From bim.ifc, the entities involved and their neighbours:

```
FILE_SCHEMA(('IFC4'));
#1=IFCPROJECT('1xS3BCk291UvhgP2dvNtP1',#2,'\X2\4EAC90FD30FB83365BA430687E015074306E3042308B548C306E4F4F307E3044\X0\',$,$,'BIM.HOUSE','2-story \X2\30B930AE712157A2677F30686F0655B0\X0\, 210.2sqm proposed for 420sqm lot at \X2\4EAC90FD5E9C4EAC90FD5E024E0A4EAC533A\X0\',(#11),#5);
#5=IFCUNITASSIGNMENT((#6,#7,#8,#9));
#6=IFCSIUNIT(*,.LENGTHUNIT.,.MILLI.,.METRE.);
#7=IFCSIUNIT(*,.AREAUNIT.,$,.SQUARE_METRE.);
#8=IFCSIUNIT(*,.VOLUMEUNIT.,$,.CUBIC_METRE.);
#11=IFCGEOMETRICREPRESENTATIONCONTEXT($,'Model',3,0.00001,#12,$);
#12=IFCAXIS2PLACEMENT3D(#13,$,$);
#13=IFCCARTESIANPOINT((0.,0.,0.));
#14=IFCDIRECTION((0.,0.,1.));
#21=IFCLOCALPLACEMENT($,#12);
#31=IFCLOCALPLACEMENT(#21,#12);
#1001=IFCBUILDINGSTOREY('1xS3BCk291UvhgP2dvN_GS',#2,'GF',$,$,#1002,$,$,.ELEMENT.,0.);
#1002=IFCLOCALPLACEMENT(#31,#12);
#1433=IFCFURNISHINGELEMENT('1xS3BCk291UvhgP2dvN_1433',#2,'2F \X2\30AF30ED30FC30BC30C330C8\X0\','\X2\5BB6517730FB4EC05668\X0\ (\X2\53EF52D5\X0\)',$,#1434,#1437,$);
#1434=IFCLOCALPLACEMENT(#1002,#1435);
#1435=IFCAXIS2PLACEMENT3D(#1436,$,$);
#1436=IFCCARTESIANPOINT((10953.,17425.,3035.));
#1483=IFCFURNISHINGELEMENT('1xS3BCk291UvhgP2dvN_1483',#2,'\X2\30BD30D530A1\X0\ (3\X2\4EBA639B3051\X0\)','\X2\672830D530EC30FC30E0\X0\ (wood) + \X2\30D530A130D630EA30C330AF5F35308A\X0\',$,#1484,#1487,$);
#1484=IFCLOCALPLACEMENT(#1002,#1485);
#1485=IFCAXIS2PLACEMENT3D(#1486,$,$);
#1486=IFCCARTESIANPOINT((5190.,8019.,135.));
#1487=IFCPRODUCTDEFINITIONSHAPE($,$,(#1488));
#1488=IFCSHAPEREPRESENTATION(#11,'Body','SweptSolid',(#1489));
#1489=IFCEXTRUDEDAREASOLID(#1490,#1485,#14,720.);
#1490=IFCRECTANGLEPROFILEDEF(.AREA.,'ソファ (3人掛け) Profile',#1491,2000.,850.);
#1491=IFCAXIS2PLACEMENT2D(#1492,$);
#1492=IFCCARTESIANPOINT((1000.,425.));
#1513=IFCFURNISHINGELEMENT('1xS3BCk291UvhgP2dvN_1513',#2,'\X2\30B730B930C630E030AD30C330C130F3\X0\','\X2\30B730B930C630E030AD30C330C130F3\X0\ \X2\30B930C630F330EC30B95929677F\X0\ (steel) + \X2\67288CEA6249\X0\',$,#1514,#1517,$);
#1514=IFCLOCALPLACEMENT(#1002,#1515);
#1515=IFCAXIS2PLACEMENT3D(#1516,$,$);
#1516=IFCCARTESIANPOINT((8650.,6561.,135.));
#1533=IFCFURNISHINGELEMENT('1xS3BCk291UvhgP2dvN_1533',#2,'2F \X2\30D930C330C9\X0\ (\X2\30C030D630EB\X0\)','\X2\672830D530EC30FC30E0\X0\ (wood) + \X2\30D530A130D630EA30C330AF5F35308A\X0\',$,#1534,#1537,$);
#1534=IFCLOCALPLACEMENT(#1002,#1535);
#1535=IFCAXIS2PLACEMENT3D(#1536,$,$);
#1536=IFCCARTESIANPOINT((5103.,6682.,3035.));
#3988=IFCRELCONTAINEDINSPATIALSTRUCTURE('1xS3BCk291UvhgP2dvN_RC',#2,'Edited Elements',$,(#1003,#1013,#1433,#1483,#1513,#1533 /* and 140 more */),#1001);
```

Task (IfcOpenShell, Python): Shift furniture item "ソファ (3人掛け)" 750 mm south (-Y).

```python
import ifcopenshell
import ifcopenshell.api.geometry
import ifcopenshell.util.placement

model = ifcopenshell.open("bim.ifc")

item = model.by_id(1483)
matrix = ifcopenshell.util.placement.get_local_placement(item.ObjectPlacement)
matrix[1, 3] -= 750.0
ifcopenshell.api.geometry.edit_object_placement(model, product=item, matrix=matrix, is_si=False)

print(ifcopenshell.util.placement.get_local_placement(item.ObjectPlacement).round(3) + 0.0)

model.write("bim_v2.ifc")
```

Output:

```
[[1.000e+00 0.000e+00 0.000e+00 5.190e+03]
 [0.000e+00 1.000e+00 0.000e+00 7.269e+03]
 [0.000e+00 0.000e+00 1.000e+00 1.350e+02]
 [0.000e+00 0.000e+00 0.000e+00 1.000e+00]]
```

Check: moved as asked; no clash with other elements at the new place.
